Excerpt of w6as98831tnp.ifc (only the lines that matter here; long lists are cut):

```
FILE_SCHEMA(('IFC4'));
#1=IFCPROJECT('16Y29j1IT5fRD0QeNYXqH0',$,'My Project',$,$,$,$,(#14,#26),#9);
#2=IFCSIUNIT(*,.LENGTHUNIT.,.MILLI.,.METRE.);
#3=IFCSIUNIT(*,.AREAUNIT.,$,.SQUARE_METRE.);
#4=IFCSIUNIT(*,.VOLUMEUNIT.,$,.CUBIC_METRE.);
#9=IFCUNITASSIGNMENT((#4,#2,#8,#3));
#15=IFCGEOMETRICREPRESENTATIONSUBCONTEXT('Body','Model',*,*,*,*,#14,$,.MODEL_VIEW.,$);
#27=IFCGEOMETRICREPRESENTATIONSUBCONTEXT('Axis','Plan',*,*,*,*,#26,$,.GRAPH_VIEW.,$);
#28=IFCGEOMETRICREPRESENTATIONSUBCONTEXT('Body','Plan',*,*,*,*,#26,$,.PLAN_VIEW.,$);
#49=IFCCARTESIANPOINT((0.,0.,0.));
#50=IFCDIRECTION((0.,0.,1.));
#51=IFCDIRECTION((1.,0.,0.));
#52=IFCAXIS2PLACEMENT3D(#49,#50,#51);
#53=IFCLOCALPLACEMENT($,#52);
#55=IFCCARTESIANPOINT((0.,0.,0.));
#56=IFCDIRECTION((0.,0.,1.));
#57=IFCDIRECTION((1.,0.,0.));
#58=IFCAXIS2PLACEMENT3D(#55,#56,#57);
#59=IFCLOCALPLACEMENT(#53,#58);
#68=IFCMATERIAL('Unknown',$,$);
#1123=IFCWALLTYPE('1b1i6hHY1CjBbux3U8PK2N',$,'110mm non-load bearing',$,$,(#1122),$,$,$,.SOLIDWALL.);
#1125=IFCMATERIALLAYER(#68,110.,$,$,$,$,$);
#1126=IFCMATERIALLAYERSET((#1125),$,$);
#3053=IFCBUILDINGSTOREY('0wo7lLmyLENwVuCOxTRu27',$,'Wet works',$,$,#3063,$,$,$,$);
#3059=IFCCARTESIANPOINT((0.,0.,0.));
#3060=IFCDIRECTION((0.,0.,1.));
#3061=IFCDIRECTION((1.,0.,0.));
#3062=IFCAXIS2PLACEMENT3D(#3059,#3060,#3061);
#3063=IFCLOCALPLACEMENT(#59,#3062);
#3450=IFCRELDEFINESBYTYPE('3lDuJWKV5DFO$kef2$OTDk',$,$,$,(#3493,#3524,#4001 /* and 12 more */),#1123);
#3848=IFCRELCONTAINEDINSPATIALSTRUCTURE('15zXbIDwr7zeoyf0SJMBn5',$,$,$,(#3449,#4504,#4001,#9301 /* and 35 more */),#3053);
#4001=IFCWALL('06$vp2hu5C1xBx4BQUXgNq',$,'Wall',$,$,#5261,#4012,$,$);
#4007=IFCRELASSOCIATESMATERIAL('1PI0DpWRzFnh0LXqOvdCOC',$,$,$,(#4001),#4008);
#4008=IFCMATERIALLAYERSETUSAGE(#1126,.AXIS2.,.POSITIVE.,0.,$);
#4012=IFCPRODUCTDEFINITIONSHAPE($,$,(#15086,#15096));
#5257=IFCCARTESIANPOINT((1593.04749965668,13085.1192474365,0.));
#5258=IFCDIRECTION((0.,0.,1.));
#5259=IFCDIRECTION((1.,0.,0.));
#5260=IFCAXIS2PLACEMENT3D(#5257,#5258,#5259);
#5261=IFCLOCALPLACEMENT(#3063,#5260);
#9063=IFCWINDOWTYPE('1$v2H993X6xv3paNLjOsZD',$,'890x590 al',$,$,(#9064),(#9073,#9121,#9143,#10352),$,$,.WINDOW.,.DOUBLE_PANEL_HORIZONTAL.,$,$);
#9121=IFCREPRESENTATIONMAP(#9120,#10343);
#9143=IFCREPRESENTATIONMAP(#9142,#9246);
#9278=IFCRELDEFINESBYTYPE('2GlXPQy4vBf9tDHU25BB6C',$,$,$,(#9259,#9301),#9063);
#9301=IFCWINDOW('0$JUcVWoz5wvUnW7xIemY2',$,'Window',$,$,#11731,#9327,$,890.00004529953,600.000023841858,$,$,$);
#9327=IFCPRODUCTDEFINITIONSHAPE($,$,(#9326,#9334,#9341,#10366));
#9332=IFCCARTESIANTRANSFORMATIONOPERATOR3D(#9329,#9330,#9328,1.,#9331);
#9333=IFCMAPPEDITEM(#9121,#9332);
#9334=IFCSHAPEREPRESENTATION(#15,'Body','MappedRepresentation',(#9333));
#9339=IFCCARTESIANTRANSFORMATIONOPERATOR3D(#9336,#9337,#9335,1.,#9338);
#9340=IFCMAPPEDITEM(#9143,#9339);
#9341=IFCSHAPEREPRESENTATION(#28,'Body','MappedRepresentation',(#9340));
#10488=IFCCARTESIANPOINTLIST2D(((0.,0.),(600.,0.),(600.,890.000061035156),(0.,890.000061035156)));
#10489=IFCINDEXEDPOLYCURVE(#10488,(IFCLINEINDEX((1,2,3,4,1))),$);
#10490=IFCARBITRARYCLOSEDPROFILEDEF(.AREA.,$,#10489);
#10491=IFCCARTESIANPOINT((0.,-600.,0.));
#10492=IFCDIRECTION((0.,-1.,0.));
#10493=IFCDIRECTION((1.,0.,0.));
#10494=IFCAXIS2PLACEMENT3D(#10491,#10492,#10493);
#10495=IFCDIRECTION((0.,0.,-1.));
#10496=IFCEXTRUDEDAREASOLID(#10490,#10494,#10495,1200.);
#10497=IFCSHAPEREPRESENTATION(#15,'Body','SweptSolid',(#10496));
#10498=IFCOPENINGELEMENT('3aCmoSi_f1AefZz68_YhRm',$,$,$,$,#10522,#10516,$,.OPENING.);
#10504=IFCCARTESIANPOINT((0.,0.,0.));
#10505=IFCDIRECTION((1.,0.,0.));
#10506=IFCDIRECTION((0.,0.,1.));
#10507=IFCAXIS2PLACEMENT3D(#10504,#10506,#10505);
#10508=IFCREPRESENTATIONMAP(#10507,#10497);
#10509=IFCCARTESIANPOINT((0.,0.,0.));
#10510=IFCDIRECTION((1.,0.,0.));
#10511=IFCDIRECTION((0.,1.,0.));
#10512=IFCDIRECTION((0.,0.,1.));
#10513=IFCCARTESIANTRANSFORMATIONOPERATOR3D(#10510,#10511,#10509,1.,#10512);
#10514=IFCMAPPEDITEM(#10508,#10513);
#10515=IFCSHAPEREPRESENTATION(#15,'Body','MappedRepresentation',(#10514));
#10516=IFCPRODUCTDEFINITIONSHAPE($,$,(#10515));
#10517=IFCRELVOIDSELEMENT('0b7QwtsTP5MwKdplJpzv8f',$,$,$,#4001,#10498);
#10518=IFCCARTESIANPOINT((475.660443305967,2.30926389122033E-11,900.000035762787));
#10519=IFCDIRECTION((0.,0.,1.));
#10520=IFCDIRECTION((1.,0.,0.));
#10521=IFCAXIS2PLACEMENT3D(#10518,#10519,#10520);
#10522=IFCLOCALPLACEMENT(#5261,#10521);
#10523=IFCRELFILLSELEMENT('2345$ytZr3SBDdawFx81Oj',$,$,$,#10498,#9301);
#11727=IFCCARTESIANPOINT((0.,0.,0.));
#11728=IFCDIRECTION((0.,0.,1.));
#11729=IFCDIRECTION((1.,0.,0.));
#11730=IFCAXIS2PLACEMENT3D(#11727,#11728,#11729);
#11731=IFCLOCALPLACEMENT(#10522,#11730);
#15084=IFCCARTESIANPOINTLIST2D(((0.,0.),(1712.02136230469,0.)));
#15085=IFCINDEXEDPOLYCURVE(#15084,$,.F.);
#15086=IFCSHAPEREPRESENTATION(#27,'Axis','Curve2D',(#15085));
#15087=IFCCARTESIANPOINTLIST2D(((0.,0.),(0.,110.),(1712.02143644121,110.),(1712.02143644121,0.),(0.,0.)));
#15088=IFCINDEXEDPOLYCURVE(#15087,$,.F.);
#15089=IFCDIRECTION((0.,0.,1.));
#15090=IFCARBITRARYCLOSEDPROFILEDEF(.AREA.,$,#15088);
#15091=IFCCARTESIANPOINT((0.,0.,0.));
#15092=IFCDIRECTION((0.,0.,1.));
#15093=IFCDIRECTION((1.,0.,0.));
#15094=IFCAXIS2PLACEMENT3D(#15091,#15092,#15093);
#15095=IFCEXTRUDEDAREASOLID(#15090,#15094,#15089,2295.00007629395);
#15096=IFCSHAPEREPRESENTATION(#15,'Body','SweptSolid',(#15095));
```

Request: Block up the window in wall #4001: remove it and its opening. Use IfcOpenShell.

```python
import ifcopenshell
import ifcopenshell.api.feature
import ifcopenshell.api.root
import ifcopenshell.geom
import ifcopenshell.util.shape

model = ifcopenshell.open("w6as98831tnp.ifc")
settings = ifcopenshell.geom.settings()


def volume(element):
    """Net volume in cubic metres, openings subtracted."""
    shape = ifcopenshell.geom.create_shape(settings, element)
    return ifcopenshell.util.shape.get_volume(shape.geometry)


window = model.by_guid("0$JUcVWoz5wvUnW7xIemY2")
opening = window.FillsVoids[0].RelatingOpeningElement
wall = opening.VoidsElements[0].RelatingBuildingElement
before = volume(wall)

ifcopenshell.api.root.remove_product(model, product=window)
ifcopenshell.api.feature.remove_feature(model, feature=opening)

after = volume(wall)

print(f"wall volume {before:.3f} -> {after:.3f} m3")

model.write("w6as98831tnp_updated.ifc")
```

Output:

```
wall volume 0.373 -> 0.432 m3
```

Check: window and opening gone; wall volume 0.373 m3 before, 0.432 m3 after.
